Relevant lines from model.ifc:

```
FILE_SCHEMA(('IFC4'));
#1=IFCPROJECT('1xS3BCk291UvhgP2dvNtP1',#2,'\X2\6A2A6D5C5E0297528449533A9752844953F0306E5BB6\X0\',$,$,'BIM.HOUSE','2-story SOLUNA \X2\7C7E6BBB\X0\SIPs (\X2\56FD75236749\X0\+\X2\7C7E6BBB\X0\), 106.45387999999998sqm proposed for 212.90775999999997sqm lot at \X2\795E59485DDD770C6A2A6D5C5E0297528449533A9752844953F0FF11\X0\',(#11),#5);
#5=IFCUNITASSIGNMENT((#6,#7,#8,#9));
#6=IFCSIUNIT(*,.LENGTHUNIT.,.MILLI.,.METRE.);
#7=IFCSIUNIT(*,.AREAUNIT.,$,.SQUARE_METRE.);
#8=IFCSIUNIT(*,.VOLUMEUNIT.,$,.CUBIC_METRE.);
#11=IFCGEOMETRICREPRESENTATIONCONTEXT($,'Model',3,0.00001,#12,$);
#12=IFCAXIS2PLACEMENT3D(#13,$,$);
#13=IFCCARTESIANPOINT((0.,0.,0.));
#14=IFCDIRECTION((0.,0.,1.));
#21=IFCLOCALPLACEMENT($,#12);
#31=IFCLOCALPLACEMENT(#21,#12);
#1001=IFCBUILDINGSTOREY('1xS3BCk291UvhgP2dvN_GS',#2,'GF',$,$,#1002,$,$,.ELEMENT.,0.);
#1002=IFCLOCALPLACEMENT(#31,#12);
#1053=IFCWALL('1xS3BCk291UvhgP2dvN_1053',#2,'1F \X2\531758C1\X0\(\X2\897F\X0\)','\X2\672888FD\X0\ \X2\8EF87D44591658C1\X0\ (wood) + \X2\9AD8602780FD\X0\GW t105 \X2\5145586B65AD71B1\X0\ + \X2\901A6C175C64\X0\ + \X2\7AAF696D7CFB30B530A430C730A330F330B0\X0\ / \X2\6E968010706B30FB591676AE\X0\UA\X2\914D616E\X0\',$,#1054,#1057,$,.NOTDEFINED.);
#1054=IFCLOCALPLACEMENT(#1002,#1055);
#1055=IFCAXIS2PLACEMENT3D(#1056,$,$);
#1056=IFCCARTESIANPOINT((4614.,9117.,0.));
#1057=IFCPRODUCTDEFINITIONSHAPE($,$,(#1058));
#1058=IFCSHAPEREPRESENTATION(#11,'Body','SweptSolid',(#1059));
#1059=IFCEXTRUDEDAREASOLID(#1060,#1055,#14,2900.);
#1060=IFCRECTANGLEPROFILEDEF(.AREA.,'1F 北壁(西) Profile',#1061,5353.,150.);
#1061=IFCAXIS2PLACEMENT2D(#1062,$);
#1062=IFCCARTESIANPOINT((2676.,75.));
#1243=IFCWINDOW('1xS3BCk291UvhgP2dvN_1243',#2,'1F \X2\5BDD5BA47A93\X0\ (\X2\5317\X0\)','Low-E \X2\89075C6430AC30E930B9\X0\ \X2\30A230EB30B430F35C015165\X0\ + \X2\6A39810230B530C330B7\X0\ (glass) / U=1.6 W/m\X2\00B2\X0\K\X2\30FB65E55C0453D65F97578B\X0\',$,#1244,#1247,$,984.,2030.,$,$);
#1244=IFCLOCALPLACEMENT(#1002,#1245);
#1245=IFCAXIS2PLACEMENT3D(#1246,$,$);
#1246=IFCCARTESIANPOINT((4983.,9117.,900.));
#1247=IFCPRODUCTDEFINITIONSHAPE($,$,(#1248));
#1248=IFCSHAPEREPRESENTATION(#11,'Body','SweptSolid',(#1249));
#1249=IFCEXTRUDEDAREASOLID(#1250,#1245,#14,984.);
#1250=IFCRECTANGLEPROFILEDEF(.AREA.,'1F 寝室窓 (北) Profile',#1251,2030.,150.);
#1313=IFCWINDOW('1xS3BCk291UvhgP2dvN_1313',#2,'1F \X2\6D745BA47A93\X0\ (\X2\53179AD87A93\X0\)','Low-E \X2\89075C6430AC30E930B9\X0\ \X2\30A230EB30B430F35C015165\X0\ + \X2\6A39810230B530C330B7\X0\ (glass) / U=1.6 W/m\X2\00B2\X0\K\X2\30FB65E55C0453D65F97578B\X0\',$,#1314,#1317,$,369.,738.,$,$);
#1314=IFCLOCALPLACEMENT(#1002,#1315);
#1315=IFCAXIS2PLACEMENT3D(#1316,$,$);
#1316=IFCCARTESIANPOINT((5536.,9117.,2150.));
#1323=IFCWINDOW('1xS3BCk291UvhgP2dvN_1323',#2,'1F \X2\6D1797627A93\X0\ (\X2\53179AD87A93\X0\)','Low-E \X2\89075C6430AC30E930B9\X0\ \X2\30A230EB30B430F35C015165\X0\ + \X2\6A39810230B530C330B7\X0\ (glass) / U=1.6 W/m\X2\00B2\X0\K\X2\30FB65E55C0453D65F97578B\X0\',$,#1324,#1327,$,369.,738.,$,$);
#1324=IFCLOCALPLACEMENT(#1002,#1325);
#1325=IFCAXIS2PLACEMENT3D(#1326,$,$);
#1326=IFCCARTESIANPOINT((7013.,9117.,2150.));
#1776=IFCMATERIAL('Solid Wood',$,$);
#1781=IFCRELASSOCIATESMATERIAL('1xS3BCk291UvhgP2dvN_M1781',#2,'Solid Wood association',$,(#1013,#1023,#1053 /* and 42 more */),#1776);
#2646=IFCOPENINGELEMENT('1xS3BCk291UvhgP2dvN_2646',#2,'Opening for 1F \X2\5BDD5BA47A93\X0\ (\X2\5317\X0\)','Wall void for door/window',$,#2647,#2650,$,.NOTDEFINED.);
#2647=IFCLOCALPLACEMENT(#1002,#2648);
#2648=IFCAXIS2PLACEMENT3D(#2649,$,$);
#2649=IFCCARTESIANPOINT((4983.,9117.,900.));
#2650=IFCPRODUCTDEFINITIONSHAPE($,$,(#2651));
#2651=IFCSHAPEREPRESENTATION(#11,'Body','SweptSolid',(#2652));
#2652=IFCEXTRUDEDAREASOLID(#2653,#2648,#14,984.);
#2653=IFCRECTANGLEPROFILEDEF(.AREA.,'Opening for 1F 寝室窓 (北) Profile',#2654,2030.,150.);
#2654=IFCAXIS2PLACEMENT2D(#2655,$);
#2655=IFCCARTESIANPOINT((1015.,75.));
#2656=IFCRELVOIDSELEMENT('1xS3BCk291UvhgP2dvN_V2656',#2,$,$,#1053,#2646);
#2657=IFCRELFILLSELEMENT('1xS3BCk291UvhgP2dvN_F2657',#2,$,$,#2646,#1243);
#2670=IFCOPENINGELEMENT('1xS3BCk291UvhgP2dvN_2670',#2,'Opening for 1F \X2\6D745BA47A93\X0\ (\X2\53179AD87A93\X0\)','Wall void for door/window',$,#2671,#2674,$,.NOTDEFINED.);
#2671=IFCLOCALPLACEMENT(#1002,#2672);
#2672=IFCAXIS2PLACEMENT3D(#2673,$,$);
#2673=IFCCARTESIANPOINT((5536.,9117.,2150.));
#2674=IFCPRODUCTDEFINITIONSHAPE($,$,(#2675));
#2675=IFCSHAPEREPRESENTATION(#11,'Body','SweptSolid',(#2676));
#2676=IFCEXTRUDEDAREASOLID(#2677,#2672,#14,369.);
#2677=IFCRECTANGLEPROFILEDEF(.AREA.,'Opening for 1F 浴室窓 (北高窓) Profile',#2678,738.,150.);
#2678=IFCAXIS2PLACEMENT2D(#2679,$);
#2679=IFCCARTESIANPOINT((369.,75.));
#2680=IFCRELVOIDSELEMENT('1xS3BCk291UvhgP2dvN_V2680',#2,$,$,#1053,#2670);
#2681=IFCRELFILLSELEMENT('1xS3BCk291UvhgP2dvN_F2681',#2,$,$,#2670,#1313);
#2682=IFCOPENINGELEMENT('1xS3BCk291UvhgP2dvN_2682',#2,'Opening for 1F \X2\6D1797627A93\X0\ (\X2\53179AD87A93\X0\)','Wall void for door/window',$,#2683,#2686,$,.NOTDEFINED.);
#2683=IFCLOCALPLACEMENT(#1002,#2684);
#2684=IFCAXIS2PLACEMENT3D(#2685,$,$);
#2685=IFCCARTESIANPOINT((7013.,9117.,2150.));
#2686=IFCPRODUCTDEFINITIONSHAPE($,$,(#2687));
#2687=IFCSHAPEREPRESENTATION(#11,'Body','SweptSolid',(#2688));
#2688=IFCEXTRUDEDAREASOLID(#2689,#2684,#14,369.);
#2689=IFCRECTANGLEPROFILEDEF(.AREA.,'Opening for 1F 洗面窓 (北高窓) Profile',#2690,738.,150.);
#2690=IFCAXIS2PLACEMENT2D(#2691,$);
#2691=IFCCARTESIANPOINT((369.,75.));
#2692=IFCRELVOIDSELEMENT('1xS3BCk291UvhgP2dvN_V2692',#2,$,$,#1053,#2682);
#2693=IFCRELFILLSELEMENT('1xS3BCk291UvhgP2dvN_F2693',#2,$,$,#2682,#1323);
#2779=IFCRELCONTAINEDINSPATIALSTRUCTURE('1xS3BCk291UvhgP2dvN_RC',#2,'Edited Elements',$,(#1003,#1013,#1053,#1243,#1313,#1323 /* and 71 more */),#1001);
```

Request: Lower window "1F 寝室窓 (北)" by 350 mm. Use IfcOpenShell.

```python
import numpy as np
import ifcopenshell
import ifcopenshell.api.geometry
import ifcopenshell.util.placement
import ifcopenshell.util.unit

model = ifcopenshell.open("model.ifc")
unit_scale = ifcopenshell.util.unit.calculate_unit_scale(model)

window = model.by_id(1243)
opening = window.FillsVoids[0].RelatingOpeningElement
dz = -0.35 / unit_scale

shift = np.array([0.0, 0.0, dz])
# The window is not placed relative to its opening, so move both.
for product in (opening, window):
    matrix = ifcopenshell.util.placement.get_local_placement(product.ObjectPlacement)
    matrix[:3, 3] += shift
    ifcopenshell.api.geometry.edit_object_placement(model, product=product, matrix=matrix, is_si=False)

print(f"moved by {dz * unit_scale:+.3f} m")

model.write("model_v2.ifc")
```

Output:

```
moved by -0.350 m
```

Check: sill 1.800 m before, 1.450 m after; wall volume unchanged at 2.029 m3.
